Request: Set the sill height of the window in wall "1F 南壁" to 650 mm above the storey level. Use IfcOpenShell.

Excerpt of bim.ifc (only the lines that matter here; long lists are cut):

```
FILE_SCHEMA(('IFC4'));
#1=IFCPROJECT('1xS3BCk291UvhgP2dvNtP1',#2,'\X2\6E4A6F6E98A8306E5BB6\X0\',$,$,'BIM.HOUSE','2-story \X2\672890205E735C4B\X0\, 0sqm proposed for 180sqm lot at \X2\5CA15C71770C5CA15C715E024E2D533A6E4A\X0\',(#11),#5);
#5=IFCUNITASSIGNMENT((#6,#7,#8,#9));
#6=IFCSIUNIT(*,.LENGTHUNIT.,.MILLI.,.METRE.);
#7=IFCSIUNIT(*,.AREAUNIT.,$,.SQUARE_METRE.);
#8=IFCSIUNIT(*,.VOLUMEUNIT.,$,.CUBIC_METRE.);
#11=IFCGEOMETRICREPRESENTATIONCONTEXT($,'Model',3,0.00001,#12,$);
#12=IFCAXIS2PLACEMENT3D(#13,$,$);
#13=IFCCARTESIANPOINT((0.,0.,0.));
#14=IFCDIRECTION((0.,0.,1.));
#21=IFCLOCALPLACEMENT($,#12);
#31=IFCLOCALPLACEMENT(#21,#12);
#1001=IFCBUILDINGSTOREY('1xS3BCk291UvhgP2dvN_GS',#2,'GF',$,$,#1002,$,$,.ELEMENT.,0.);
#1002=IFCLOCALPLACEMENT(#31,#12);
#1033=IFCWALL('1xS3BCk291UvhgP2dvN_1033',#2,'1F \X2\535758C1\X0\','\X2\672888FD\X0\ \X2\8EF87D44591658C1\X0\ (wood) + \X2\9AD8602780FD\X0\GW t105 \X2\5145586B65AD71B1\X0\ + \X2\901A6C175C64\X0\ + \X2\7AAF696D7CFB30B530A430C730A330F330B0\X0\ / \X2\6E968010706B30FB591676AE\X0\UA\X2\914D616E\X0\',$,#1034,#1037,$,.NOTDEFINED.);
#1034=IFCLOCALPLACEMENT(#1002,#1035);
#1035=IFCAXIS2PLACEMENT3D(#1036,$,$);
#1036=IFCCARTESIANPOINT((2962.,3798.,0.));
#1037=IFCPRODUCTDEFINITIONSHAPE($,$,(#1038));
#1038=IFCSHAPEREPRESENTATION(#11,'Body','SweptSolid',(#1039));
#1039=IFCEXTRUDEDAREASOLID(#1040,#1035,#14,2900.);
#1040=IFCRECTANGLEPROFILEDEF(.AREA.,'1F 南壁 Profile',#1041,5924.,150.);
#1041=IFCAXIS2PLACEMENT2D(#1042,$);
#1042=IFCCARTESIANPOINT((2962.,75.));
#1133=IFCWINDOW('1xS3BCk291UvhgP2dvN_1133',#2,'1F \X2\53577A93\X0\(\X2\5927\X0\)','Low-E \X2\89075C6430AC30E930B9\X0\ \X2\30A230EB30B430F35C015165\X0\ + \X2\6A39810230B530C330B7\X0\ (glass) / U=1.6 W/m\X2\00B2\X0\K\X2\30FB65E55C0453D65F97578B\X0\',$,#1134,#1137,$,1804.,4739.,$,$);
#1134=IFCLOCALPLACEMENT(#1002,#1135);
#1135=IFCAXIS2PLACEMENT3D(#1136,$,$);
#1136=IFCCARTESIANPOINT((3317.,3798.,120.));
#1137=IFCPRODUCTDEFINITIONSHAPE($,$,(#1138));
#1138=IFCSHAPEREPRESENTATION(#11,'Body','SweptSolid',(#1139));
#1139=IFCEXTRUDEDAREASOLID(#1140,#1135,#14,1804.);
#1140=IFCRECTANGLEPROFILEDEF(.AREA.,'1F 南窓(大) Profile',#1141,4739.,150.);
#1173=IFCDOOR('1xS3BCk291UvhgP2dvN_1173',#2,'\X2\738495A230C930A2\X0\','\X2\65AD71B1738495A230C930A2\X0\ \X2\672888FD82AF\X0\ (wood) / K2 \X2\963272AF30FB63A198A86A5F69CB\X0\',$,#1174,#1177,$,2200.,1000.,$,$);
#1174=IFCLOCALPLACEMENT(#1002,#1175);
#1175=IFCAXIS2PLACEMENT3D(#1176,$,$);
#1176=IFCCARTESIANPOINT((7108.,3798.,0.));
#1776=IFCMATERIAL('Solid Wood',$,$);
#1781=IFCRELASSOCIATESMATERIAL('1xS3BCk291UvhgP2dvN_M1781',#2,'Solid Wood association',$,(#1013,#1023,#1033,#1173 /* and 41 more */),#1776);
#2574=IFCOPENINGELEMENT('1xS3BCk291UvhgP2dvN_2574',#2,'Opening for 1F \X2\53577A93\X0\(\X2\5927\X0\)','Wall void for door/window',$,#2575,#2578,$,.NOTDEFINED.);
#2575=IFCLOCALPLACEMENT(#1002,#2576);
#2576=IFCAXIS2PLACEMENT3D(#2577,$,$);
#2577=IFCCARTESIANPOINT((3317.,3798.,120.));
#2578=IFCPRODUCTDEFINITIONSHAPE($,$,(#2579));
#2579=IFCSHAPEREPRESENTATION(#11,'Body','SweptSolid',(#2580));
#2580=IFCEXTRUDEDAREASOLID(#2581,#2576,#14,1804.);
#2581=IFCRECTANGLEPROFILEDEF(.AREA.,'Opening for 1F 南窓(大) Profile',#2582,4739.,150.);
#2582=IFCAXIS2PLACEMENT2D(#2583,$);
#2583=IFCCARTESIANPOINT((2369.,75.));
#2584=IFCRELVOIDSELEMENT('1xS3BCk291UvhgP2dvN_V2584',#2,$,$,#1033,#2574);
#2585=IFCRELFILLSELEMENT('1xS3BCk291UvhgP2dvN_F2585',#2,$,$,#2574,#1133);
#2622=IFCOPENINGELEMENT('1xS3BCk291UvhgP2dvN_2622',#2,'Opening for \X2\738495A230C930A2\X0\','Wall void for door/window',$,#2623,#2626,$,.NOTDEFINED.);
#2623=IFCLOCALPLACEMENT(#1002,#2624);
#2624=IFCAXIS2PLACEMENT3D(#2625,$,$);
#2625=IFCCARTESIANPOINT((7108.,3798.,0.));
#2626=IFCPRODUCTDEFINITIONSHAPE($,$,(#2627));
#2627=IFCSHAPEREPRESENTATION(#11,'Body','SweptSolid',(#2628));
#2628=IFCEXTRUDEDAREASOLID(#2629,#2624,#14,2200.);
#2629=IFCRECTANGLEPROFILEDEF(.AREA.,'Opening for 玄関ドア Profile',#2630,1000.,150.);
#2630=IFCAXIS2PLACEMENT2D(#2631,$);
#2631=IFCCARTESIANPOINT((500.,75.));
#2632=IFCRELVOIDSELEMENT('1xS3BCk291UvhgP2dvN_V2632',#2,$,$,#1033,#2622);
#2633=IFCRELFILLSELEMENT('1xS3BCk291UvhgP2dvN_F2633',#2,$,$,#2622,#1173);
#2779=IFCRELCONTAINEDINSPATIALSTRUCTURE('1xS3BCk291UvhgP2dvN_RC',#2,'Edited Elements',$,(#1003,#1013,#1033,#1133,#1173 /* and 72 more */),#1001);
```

```python
import numpy as np
import ifcopenshell
import ifcopenshell.api.geometry
import ifcopenshell.geom
import ifcopenshell.util.element
import ifcopenshell.util.placement
import ifcopenshell.util.shape
import ifcopenshell.util.unit

model = ifcopenshell.open("bim.ifc")
unit_scale = ifcopenshell.util.unit.calculate_unit_scale(model)

window = model.by_guid("1xS3BCk291UvhgP2dvN_1133")
opening = window.FillsVoids[0].RelatingOpeningElement
storey = ifcopenshell.util.element.get_container(window, ifc_class="IfcBuildingStorey")
level = ifcopenshell.util.placement.get_local_placement(storey.ObjectPlacement)[2, 3]

# The opening's origin need not be at the sill, so measure its lowest point.
shape = ifcopenshell.geom.create_shape(ifcopenshell.geom.settings(), opening)
bottom = ifcopenshell.util.shape.get_shape_bottom_elevation(shape, shape.geometry) / unit_scale
dz = level + 650.0 - bottom

shift = np.array([0.0, 0.0, dz])
# The window is not placed relative to its opening, so move both.
for product in (opening, window):
    matrix = ifcopenshell.util.placement.get_local_placement(product.ObjectPlacement)
    matrix[:3, 3] += shift
    ifcopenshell.api.geometry.edit_object_placement(model, product=product, matrix=matrix, is_si=False)

print(f"moved by {dz * unit_scale:+.3f} m")

model.write("bim_updated.ifc")
```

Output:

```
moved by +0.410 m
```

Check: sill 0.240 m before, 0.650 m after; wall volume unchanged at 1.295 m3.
